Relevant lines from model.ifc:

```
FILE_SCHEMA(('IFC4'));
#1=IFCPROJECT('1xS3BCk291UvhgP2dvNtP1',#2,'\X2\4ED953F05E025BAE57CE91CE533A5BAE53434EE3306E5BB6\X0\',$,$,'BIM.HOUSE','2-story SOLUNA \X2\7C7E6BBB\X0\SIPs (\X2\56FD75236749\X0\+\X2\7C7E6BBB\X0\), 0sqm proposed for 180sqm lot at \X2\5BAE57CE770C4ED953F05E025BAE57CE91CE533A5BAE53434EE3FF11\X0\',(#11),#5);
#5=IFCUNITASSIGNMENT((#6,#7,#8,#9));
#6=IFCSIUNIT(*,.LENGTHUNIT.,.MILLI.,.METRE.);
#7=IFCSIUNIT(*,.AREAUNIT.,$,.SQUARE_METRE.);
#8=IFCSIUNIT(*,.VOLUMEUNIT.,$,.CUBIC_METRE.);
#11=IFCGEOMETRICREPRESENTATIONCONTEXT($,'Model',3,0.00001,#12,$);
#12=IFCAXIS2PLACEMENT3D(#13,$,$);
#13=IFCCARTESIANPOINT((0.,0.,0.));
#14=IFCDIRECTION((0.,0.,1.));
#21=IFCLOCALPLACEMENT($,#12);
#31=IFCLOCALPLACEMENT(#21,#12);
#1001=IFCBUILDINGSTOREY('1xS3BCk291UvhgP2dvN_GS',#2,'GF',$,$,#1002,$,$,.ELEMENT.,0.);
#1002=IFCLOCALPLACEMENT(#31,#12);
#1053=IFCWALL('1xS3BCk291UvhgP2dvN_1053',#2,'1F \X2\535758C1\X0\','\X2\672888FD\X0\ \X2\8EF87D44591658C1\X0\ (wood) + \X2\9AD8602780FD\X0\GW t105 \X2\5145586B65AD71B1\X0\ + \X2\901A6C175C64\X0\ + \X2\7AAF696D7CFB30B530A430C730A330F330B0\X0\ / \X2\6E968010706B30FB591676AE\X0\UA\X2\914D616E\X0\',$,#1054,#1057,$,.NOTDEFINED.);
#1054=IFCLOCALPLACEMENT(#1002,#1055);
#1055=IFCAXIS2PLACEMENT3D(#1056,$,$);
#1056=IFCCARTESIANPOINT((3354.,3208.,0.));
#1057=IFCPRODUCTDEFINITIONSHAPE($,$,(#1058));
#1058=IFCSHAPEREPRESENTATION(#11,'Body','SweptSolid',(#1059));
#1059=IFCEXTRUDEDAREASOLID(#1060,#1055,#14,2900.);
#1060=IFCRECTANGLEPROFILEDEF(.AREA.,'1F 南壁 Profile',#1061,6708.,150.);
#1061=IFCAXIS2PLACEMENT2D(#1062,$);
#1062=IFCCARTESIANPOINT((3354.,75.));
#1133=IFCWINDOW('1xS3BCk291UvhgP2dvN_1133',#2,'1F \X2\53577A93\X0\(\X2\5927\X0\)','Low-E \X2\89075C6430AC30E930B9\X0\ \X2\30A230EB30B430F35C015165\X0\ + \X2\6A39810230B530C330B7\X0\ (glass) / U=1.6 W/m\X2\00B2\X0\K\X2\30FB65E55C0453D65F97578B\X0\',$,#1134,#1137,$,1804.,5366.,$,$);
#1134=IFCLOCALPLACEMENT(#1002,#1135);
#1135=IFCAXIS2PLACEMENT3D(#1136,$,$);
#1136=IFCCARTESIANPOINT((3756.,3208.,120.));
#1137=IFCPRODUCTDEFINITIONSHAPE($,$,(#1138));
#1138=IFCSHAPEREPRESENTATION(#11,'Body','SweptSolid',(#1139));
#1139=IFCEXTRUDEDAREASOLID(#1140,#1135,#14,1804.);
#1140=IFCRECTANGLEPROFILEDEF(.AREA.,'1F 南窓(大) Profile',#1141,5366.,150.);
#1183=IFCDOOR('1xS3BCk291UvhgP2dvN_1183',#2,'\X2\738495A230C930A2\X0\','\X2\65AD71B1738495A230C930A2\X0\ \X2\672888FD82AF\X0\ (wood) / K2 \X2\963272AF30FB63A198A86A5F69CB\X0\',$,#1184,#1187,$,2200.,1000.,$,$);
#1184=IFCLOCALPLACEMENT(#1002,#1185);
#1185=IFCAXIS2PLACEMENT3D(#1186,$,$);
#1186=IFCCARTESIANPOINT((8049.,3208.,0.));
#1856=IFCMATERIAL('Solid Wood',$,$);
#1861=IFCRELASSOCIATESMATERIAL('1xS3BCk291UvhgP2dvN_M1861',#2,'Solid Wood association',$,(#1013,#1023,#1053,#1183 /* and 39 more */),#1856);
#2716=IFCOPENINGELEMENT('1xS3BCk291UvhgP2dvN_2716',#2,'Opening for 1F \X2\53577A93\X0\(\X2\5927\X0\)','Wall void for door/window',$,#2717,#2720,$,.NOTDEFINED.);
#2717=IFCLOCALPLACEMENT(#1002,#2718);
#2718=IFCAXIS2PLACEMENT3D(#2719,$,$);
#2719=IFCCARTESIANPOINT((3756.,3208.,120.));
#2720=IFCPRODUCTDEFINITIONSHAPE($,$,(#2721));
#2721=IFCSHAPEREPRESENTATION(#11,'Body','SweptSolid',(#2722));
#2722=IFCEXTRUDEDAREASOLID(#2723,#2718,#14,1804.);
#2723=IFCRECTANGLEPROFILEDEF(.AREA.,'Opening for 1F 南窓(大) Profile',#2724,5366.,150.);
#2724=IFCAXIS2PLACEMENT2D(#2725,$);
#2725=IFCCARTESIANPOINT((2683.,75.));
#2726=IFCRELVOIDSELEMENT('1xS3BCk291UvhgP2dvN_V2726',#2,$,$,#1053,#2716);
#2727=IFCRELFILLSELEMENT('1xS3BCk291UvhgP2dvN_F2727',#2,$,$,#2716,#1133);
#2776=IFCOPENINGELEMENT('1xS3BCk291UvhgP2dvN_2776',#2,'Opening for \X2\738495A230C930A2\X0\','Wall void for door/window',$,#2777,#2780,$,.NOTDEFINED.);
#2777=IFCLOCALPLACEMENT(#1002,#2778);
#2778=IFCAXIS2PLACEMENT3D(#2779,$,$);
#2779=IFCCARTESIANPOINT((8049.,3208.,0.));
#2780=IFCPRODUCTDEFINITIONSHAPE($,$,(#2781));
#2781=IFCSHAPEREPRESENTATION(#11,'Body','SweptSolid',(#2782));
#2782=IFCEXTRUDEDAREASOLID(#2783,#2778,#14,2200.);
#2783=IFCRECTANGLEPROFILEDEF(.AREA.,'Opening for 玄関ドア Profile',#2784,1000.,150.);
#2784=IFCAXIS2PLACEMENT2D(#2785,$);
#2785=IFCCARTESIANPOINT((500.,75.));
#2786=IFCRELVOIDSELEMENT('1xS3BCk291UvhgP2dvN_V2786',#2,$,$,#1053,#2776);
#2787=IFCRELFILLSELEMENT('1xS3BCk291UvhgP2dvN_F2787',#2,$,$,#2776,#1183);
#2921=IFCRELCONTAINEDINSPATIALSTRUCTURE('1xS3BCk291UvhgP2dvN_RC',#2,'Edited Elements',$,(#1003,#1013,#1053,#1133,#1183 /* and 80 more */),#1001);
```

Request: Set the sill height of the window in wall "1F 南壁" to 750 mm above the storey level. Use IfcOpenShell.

```python
import numpy as np
import ifcopenshell
import ifcopenshell.api.geometry
import ifcopenshell.geom
import ifcopenshell.util.element
import ifcopenshell.util.placement
import ifcopenshell.util.shape
import ifcopenshell.util.unit

model = ifcopenshell.open("model.ifc")
unit_scale = ifcopenshell.util.unit.calculate_unit_scale(model)

window = model.by_guid("1xS3BCk291UvhgP2dvN_1133")
opening = window.FillsVoids[0].RelatingOpeningElement
storey = ifcopenshell.util.element.get_container(window, ifc_class="IfcBuildingStorey")
level = ifcopenshell.util.placement.get_local_placement(storey.ObjectPlacement)[2, 3]

# The opening's origin need not be at the sill, so measure its lowest point.
shape = ifcopenshell.geom.create_shape(ifcopenshell.geom.settings(), opening)
bottom = ifcopenshell.util.shape.get_shape_bottom_elevation(shape, shape.geometry) / unit_scale
dz = level + 0.75 / unit_scale - bottom

shift = np.array([0.0, 0.0, dz])
# The window is not placed relative to its opening, so move both.
for product in (opening, window):
    matrix = ifcopenshell.util.placement.get_local_placement(product.ObjectPlacement)
    matrix[:3, 3] += shift
    ifcopenshell.api.geometry.edit_object_placement(model, product=product, matrix=matrix, is_si=False)

print(f"moved by {dz * unit_scale:+.3f} m")

model.write("model_v2.ifc")
```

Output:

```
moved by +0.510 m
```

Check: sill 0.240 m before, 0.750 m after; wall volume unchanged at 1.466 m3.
